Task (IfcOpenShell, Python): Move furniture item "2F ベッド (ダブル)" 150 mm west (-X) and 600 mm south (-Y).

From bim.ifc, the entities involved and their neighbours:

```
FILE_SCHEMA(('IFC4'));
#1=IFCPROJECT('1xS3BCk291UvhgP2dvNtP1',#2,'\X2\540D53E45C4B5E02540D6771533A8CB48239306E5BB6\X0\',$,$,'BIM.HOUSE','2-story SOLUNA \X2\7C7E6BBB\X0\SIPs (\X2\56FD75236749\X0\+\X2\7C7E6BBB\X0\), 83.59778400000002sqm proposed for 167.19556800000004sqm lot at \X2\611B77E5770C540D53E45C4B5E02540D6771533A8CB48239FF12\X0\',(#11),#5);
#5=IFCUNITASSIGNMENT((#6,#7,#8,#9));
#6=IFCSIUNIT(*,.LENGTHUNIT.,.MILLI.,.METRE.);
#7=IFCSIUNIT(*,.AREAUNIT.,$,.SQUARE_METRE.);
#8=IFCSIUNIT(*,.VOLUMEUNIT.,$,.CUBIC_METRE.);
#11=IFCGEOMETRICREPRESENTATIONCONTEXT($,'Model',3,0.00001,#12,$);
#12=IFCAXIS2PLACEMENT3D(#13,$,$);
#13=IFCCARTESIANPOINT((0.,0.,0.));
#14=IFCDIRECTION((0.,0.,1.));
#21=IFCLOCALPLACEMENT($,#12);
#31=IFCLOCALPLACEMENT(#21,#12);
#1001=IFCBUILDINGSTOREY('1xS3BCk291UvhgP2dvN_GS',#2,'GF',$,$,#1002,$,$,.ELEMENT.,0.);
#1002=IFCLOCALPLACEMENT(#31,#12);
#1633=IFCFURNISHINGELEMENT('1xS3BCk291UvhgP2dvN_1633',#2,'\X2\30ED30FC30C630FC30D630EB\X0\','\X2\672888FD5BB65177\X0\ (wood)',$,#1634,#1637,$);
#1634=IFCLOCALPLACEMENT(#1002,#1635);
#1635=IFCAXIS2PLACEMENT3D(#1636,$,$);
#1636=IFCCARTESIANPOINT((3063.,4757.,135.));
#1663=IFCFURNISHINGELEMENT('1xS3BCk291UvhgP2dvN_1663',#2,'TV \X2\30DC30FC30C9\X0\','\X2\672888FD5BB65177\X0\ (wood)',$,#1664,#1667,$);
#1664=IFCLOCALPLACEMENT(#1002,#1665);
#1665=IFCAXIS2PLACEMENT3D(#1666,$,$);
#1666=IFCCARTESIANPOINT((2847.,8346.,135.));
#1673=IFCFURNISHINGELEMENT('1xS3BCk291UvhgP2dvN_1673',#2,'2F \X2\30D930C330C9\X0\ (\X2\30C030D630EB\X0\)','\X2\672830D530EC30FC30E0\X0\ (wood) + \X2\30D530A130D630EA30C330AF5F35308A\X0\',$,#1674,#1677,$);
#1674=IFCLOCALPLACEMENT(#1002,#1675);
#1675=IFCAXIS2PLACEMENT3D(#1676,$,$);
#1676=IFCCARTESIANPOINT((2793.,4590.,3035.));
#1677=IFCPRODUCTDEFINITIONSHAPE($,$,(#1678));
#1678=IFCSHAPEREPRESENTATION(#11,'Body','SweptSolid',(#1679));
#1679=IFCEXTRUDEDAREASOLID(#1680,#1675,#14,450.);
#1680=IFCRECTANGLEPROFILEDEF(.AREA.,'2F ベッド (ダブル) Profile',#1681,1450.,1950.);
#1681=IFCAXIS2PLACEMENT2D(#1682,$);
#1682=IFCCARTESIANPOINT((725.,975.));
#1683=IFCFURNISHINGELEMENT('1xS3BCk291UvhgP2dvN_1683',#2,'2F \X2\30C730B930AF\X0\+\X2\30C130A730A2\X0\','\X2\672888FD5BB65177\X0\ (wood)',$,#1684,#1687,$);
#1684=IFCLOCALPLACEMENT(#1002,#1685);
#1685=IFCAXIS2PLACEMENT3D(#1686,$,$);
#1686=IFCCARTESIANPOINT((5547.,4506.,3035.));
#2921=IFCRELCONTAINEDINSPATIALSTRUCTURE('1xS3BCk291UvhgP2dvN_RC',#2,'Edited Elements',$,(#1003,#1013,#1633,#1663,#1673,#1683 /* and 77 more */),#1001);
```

```python
import ifcopenshell
import ifcopenshell.api.geometry
import ifcopenshell.util.placement
import ifcopenshell.util.unit

model = ifcopenshell.open("bim.ifc")
unit_scale = ifcopenshell.util.unit.calculate_unit_scale(model)

item = model.by_guid("1xS3BCk291UvhgP2dvN_1673")
matrix = ifcopenshell.util.placement.get_local_placement(item.ObjectPlacement)
matrix[0, 3] -= 0.15 / unit_scale
matrix[1, 3] -= 0.6 / unit_scale
ifcopenshell.api.geometry.edit_object_placement(model, product=item, matrix=matrix, is_si=False)

print(ifcopenshell.util.placement.get_local_placement(item.ObjectPlacement).round(3) + 0.0)

model.write("bim_updated.ifc")
```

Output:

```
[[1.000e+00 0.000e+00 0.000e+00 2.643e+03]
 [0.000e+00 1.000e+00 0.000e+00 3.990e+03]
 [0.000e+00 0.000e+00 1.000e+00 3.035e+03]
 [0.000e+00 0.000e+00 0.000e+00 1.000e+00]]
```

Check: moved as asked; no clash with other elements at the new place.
